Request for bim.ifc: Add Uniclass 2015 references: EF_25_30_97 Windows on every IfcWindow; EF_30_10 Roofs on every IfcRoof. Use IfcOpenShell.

First a look at what the model holds.

```python
import ifcopenshell

model = ifcopenshell.open("bim.ifc")
print(model.schema)
print("classifications:", [c.Name for c in model.by_type("IfcClassification")])
for ifc_class in ("IfcDoor", "IfcRoof", "IfcStair", "IfcWall", "IfcWindow"):
    print(ifc_class, len(model.by_type(ifc_class)))
```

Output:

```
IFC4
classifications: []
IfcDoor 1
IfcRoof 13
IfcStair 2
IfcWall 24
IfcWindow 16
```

```python
import ifcopenshell
import ifcopenshell.api.classification

model = ifcopenshell.open("bim.ifc")

system = ifcopenshell.api.classification.add_classification(model, classification="Uniclass 2015")

codes = {
    "IfcWindow": ("EF_25_30_97", "Windows"),
    "IfcRoof": ("EF_30_10", "Roofs"),
}
for ifc_class, (code, name) in codes.items():
    products = model.by_type(ifc_class)
    ifcopenshell.api.classification.add_reference(
        model, products=products, classification=system, identification=code, name=name
    )
    print(code, len(products))

model.write("bim_edited.ifc")
```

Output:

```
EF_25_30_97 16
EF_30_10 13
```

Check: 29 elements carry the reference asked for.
